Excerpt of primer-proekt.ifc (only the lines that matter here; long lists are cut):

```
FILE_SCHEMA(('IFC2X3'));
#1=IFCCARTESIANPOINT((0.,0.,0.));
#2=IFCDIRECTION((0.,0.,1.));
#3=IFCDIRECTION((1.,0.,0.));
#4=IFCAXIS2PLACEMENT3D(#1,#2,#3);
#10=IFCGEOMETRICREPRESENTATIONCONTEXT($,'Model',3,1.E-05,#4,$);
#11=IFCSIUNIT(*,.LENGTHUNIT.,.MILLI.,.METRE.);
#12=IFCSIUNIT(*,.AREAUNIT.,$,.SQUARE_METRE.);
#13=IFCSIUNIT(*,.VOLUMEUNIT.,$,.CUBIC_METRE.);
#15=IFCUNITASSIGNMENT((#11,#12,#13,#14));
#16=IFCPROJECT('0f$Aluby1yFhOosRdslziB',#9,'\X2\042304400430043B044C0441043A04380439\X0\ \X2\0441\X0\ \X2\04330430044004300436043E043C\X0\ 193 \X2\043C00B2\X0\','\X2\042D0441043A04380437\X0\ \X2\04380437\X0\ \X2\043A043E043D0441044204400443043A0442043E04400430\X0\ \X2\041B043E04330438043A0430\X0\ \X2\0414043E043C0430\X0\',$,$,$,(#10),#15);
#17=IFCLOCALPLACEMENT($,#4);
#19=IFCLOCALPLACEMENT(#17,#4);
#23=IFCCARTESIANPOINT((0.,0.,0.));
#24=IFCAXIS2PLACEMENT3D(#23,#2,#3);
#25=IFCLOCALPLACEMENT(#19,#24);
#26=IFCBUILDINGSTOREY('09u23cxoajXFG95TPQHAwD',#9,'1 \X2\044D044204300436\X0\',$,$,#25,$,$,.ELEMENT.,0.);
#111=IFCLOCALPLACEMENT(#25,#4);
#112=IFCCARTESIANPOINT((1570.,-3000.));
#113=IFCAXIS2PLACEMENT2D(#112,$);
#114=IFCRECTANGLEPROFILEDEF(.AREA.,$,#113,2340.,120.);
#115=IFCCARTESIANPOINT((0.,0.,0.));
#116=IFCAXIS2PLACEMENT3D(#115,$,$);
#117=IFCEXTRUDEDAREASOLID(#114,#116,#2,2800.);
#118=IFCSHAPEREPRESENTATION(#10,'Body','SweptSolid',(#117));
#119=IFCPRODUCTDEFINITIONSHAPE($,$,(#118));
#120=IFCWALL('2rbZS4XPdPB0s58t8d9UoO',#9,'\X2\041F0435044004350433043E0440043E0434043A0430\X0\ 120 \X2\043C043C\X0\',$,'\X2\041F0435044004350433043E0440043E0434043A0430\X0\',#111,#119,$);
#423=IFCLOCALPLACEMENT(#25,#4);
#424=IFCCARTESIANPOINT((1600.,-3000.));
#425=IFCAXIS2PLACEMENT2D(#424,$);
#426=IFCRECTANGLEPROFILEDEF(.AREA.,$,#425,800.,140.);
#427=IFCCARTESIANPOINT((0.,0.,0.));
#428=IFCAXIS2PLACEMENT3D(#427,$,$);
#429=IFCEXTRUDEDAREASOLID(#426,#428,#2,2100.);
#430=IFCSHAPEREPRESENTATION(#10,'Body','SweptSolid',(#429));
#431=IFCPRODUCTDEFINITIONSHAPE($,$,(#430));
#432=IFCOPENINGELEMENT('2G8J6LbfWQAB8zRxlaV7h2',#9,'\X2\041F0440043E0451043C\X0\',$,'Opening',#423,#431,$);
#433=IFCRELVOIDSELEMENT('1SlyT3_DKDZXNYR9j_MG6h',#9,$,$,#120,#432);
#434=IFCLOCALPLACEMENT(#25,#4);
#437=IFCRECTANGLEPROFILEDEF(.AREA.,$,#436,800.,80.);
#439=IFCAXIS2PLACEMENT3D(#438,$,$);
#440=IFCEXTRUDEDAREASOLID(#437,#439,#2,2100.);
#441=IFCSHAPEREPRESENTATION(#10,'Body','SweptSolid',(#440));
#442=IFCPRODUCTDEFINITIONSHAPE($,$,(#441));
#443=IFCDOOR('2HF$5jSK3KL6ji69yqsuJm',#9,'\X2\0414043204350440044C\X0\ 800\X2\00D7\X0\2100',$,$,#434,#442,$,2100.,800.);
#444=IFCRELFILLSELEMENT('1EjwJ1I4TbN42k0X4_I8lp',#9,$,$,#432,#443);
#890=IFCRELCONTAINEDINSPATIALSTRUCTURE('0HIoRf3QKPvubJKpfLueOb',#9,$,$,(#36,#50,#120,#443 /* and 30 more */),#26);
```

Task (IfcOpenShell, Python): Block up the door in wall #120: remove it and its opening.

```python
import ifcopenshell
import ifcopenshell.api.feature
import ifcopenshell.api.root
import ifcopenshell.geom
import ifcopenshell.util.shape

model = ifcopenshell.open("primer-proekt.ifc")
settings = ifcopenshell.geom.settings()


def volume(element):
    """Net volume in cubic metres, openings subtracted."""
    shape = ifcopenshell.geom.create_shape(settings, element)
    return ifcopenshell.util.shape.get_volume(shape.geometry)


door = model.by_guid("2HF$5jSK3KL6ji69yqsuJm")
opening = door.FillsVoids[0].RelatingOpeningElement
wall = opening.VoidsElements[0].RelatingBuildingElement
before = volume(wall)

ifcopenshell.api.root.remove_product(model, product=door)
ifcopenshell.api.feature.remove_feature(model, feature=opening)

after = volume(wall)

print(f"wall volume {before:.3f} -> {after:.3f} m3")

model.write("primer-proekt_edited.ifc")
```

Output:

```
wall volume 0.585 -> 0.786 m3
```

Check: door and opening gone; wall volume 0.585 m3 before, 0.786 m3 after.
